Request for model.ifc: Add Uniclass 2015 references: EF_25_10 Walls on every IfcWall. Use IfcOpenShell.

First a look at what the model holds.

```python
import ifcopenshell

model = ifcopenshell.open("model.ifc")
print(model.schema)
print("classifications:", [c.Name for c in model.by_type("IfcClassification")])
for ifc_class in ("IfcDoor", "IfcRoof", "IfcStair", "IfcWall", "IfcWindow"):
    print(ifc_class, len(model.by_type(ifc_class)))
```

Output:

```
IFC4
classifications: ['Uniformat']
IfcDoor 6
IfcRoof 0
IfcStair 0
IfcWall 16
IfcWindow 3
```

```python
import ifcopenshell
import ifcopenshell.api.classification

model = ifcopenshell.open("model.ifc")

system = ifcopenshell.api.classification.add_classification(model, classification="Uniclass 2015")

codes = {
    "IfcWall": ("EF_25_10", "Walls"),
}
for ifc_class, (code, name) in codes.items():
    products = model.by_type(ifc_class)
    ifcopenshell.api.classification.add_reference(
        model, products=products, classification=system, identification=code, name=name
    )
    print(code, len(products))

model.write("model_edited.ifc")
```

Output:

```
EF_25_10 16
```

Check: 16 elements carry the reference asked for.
